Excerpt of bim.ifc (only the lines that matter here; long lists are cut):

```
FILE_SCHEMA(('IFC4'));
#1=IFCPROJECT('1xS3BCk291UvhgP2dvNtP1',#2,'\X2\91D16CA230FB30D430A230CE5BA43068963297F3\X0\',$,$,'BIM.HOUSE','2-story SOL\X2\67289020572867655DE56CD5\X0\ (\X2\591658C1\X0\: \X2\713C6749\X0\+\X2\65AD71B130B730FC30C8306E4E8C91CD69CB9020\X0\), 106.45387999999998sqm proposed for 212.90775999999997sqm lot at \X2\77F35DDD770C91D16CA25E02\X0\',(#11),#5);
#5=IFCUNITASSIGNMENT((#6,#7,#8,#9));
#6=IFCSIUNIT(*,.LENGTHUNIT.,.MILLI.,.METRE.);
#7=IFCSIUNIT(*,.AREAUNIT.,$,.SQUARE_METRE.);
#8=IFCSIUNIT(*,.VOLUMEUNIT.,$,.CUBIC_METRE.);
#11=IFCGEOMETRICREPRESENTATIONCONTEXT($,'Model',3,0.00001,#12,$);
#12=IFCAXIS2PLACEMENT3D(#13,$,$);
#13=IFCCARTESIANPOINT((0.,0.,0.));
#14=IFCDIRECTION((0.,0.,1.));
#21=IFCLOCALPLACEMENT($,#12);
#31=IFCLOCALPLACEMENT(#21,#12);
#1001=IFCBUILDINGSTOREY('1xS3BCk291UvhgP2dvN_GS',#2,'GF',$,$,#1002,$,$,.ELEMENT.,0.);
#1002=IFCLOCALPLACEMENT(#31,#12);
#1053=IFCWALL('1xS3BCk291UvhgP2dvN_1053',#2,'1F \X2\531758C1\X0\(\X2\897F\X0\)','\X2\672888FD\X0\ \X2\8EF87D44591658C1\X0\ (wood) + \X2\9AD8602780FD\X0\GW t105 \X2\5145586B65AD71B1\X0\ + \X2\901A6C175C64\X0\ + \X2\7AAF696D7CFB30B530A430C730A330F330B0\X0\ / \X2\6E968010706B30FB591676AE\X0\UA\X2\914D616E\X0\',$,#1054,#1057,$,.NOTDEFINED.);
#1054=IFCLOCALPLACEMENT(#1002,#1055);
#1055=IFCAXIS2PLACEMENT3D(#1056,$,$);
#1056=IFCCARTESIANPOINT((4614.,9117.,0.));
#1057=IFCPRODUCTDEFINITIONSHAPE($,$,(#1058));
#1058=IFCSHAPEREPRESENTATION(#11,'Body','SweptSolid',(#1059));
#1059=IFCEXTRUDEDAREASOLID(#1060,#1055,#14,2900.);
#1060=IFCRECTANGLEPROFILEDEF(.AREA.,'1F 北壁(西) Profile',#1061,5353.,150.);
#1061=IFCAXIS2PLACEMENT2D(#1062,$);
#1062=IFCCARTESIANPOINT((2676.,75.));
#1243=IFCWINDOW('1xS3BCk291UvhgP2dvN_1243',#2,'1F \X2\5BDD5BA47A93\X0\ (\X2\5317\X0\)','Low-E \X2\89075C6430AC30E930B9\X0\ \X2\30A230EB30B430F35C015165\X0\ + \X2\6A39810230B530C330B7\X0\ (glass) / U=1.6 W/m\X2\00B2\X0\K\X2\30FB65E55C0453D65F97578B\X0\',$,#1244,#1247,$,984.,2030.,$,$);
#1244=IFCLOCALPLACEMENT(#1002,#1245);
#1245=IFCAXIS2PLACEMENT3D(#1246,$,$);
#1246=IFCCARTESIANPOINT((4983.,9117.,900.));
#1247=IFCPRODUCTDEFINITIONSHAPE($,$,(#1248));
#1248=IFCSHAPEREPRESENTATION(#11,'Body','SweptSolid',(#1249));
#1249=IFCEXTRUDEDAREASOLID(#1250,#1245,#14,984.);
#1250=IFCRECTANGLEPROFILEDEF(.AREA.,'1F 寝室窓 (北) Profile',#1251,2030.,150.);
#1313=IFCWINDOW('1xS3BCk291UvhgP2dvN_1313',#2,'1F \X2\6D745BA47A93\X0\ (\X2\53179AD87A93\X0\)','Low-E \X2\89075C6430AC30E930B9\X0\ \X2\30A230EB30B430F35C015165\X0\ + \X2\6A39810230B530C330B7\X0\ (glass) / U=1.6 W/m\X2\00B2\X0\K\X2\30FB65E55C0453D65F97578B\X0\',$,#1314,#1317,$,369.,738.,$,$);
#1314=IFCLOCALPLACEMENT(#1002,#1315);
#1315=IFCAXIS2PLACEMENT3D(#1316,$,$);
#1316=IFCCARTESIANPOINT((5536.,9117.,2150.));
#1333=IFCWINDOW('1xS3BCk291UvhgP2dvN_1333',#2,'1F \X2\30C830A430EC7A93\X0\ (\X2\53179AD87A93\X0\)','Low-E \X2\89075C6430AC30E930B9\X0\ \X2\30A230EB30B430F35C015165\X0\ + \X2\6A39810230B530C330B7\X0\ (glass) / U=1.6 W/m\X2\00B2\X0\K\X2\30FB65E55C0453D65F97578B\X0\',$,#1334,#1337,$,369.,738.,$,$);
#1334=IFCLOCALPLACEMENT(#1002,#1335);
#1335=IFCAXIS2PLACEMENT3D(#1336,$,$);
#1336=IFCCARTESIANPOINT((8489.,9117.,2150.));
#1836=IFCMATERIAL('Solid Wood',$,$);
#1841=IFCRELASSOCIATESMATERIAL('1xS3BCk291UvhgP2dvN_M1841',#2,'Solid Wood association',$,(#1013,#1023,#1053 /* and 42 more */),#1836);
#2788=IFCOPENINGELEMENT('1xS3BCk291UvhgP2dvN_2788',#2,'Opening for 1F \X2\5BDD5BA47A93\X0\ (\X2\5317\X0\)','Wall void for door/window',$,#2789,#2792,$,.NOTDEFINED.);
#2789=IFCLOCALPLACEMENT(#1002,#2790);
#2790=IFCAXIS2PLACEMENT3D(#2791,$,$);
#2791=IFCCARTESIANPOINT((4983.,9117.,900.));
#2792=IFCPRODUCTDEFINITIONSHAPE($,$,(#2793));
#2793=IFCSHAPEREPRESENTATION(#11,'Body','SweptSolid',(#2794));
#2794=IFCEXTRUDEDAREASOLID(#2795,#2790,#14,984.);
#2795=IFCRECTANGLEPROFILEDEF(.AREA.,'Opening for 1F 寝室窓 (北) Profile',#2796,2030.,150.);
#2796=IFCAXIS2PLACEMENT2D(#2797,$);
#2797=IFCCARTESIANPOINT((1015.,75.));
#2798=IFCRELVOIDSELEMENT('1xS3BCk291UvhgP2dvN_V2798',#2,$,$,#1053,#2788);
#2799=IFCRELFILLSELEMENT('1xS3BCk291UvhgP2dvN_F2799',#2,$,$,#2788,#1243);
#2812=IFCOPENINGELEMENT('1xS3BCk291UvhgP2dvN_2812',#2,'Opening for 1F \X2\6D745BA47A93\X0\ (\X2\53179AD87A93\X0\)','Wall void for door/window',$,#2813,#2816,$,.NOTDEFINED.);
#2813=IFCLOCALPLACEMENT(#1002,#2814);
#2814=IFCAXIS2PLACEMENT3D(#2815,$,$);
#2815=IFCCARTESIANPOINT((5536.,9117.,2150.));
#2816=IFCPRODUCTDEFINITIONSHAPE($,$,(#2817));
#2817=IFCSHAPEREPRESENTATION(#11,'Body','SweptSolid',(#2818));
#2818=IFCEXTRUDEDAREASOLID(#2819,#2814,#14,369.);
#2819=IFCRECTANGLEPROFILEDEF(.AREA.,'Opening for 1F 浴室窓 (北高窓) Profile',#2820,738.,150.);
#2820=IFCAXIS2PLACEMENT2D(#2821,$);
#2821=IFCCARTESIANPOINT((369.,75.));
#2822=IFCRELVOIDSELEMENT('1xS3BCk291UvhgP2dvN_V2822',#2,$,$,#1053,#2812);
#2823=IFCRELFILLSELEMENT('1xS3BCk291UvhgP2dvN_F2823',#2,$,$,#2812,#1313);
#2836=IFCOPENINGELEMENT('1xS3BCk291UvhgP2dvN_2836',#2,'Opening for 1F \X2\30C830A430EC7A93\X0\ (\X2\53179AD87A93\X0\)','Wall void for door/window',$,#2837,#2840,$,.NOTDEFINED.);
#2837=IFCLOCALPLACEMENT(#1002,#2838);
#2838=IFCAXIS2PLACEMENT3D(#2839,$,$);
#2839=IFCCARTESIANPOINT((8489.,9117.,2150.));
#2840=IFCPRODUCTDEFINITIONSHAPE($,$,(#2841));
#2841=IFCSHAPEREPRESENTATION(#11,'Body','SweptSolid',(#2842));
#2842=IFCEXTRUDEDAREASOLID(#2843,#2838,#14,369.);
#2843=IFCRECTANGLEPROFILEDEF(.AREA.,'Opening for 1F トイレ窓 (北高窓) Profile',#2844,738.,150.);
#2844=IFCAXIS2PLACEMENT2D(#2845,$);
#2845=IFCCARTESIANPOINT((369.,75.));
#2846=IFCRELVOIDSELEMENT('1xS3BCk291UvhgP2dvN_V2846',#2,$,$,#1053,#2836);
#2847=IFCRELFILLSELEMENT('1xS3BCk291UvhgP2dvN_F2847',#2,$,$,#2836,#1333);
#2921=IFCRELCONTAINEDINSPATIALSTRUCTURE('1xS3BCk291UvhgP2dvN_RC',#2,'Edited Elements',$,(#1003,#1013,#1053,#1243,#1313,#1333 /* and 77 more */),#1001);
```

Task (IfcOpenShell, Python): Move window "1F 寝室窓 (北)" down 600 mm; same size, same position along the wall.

```python
import numpy as np
import ifcopenshell
import ifcopenshell.api.geometry
import ifcopenshell.util.placement
import ifcopenshell.util.unit

model = ifcopenshell.open("bim.ifc")
unit_scale = ifcopenshell.util.unit.calculate_unit_scale(model)

window = model.by_id(1243)
opening = window.FillsVoids[0].RelatingOpeningElement
dz = -600.0

shift = np.array([0.0, 0.0, dz])
# The window is not placed relative to its opening, so move both.
for product in (opening, window):
    matrix = ifcopenshell.util.placement.get_local_placement(product.ObjectPlacement)
    matrix[:3, 3] += shift
    ifcopenshell.api.geometry.edit_object_placement(model, product=product, matrix=matrix, is_si=False)

print(f"moved by {dz * unit_scale:+.3f} m")

model.write("bim-out.ifc")
```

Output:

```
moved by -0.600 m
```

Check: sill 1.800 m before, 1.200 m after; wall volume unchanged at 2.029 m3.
